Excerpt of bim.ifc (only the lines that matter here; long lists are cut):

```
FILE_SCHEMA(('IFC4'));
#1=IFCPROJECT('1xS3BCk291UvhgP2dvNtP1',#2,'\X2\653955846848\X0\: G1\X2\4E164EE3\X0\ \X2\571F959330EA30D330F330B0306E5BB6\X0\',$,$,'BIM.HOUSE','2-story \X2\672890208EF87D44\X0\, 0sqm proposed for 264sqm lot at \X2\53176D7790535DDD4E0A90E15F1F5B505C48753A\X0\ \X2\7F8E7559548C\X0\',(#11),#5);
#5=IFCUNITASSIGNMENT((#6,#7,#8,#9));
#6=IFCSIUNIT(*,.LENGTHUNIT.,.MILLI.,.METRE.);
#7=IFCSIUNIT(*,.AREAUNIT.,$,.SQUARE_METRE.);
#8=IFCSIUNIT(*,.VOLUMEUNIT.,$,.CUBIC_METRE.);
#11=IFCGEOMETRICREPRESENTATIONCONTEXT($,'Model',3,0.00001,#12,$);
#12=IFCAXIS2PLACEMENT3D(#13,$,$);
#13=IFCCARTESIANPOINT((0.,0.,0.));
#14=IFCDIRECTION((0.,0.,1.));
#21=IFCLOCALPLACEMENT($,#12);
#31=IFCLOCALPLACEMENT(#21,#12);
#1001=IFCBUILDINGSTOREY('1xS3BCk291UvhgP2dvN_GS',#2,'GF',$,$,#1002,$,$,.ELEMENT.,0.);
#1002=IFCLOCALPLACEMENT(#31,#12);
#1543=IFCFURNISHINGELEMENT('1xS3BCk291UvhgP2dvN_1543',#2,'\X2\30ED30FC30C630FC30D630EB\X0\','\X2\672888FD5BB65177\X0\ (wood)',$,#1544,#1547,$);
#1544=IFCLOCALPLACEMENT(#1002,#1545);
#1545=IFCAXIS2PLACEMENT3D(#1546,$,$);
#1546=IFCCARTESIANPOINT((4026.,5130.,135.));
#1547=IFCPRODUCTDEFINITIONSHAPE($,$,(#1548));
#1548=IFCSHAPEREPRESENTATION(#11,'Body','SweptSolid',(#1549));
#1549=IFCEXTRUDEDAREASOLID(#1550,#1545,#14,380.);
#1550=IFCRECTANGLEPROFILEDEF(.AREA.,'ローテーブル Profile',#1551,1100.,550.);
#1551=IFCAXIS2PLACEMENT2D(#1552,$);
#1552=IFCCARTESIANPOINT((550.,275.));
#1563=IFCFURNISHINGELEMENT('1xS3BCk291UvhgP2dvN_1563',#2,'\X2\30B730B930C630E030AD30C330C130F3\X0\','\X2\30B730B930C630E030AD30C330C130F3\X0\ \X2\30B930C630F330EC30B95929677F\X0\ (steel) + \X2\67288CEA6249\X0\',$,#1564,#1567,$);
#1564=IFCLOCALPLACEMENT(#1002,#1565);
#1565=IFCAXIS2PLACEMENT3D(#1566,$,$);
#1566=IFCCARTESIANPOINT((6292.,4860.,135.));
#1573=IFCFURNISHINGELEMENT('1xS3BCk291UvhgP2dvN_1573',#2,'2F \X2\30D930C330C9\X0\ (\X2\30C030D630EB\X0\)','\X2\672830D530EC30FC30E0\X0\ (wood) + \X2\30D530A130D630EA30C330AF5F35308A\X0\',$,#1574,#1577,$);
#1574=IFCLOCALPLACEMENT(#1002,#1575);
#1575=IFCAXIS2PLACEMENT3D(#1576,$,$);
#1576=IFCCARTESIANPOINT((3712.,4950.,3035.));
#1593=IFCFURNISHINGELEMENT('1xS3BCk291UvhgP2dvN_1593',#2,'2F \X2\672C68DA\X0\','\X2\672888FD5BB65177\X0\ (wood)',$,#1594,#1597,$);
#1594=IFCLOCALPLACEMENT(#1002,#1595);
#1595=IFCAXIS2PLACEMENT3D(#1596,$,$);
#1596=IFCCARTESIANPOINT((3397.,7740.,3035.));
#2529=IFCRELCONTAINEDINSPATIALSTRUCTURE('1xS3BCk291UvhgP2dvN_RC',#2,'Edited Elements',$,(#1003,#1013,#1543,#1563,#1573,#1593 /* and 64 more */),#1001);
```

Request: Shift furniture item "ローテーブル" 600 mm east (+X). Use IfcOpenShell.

```python
import ifcopenshell
import ifcopenshell.api.geometry
import ifcopenshell.util.placement

model = ifcopenshell.open("bim.ifc")

item = model.by_id(1543)
matrix = ifcopenshell.util.placement.get_local_placement(item.ObjectPlacement)
matrix[0, 3] += 600.0
ifcopenshell.api.geometry.edit_object_placement(model, product=item, matrix=matrix, is_si=False)

print(ifcopenshell.util.placement.get_local_placement(item.ObjectPlacement).round(3) + 0.0)

model.write("bim-out.ifc")
```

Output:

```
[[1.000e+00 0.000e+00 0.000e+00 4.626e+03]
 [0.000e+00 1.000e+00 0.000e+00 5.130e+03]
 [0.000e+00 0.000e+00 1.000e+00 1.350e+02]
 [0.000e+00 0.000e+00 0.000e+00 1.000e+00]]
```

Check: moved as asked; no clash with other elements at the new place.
